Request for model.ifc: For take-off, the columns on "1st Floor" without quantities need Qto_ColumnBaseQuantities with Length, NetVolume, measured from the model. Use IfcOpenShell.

First a look at what the model holds.

```python
import ifcopenshell
import ifcopenshell.util.element
import ifcopenshell.util.unit

model = ifcopenshell.open("model.ifc")
print(model.schema)
for unit_type in ("LENGTHUNIT", "AREAUNIT", "VOLUMEUNIT"):
    print(unit_type, ifcopenshell.util.unit.calculate_unit_scale(model, unit_type))
storey = next(s for s in model.by_type("IfcBuildingStorey") if s.Name == "1st Floor")
columns = [e for e in ifcopenshell.util.element.get_decomposition(storey) if e.is_a("IfcColumn")]
for e in sorted(columns, key=lambda e: e.id()):
    print(e.id(), e.is_a(), e.Name, list(ifcopenshell.util.element.get_psets(e, qtos_only=True)), sep=" | ")
```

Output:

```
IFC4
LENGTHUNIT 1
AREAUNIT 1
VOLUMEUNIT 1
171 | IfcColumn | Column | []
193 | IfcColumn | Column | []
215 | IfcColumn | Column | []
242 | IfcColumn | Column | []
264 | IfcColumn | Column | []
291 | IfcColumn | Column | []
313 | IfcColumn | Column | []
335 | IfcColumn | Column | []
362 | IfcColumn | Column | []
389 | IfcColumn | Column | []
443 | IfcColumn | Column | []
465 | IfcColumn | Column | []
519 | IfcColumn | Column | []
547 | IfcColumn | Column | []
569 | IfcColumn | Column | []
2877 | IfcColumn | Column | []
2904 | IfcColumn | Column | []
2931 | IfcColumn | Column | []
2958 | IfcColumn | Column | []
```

```python
import ifcopenshell
import ifcopenshell.api.pset
import ifcopenshell.geom
import ifcopenshell.util.element
import ifcopenshell.util.shape
import ifcopenshell.util.unit

model = ifcopenshell.open("model.ifc")
unit_scale = ifcopenshell.util.unit.calculate_unit_scale(model)
volume_scale = ifcopenshell.util.unit.calculate_unit_scale(model, "VOLUMEUNIT")
settings = ifcopenshell.geom.settings()

storey = next(s for s in model.by_type("IfcBuildingStorey") if s.Name == "1st Floor")
columns = [e for e in ifcopenshell.util.element.get_decomposition(storey) if e.is_a("IfcColumn")]

for e in sorted(columns, key=lambda e: e.id()):
    if ifcopenshell.util.element.get_psets(e, qtos_only=True, should_inherit=False):
        continue
    # Geometry comes back in metres, in the element's own axes.
    shape = ifcopenshell.geom.create_shape(settings, e)
    values = {
        "Length": ifcopenshell.util.shape.get_z(shape.geometry) / unit_scale,
        "NetVolume": ifcopenshell.util.shape.get_volume(shape.geometry) / volume_scale,
    }
    qto = ifcopenshell.api.pset.add_qto(model, product=e, name="Qto_ColumnBaseQuantities")
    ifcopenshell.api.pset.edit_qto(model, qto=qto, properties=values)
    print(e.id(), {k: round(v, 3) for k, v in values.items()})

model.write("model_updated.ifc")
```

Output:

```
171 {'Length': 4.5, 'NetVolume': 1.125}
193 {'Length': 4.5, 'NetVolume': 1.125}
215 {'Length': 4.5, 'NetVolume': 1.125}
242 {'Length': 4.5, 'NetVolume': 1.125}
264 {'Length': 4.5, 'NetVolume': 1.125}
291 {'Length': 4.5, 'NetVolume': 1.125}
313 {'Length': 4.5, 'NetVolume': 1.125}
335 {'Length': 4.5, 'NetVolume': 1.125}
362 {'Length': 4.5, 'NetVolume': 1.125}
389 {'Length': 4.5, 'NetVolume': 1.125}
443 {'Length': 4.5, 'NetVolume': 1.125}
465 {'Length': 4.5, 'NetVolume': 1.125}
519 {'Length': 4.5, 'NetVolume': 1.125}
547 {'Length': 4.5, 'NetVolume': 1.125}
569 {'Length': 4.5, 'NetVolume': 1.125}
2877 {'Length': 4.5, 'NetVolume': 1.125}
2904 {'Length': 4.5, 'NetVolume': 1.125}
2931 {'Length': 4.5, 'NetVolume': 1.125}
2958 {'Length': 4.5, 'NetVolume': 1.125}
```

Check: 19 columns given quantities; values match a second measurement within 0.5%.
